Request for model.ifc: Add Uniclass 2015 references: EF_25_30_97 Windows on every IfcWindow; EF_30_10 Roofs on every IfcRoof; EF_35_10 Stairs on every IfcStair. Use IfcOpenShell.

First a look at what the model holds.

```python
import ifcopenshell

model = ifcopenshell.open("model.ifc")
print(model.schema)
print("classifications:", [c.Name for c in model.by_type("IfcClassification")])
for ifc_class in ("IfcDoor", "IfcRoof", "IfcStair", "IfcWall", "IfcWindow"):
    print(ifc_class, len(model.by_type(ifc_class)))
```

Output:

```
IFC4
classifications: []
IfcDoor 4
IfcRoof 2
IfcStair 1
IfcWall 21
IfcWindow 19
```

```python
import ifcopenshell
import ifcopenshell.api.classification

model = ifcopenshell.open("model.ifc")

system = ifcopenshell.api.classification.add_classification(model, classification="Uniclass 2015")

codes = {
    "IfcWindow": ("EF_25_30_97", "Windows"),
    "IfcRoof": ("EF_30_10", "Roofs"),
    "IfcStair": ("EF_35_10", "Stairs"),
}
for ifc_class, (code, name) in codes.items():
    products = model.by_type(ifc_class)
    ifcopenshell.api.classification.add_reference(
        model, products=products, classification=system, identification=code, name=name
    )
    print(code, len(products))

model.write("model_v2.ifc")
```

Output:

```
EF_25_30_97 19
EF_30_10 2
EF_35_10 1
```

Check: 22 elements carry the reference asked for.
